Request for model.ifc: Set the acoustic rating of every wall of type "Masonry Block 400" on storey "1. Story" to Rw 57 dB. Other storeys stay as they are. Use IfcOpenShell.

First a look at what the model holds.

```python
import ifcopenshell
import ifcopenshell.util.element

model = ifcopenshell.open("model.ifc")
print(model.schema)
storey = next(s for s in model.by_type("IfcBuildingStorey") if s.Name == "1. Story")
walls = [e for e in ifcopenshell.util.element.get_decomposition(storey) if e.is_a("IfcWall")]
seen = {}
for e in walls:
    element_type = ifcopenshell.util.element.get_type(e)
    key = (element_type.Name if element_type != e and element_type else None, ifcopenshell.util.element.get_pset(e, "Pset_WallCommon", "AcousticRating"))
    seen[key] = seen.get(key, 0) + 1
for (name, value), count in sorted(seen.items(), key=str):
    print(count, "x", name, "|", value)
```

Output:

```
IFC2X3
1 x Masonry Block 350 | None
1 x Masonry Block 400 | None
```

```python
import ifcopenshell
import ifcopenshell.api.pset
import ifcopenshell.util.element

model = ifcopenshell.open("model.ifc")

storey = next(s for s in model.by_type("IfcBuildingStorey") if s.Name == "1. Story")
walls = [e for e in ifcopenshell.util.element.get_decomposition(storey) if e.is_a("IfcWall")]

count = 0
for e in walls:
    element_type = ifcopenshell.util.element.get_type(e)
    if element_type in (None, e) or element_type.Name != "Masonry Block 400":
        continue
    # add_pset returns the element's existing set when there is one.
    pset = ifcopenshell.api.pset.add_pset(model, product=e, name="Pset_WallCommon")
    ifcopenshell.api.pset.edit_pset(model, pset=pset, properties={"AcousticRating": "Rw 57 dB"})
    count += 1

print(count, "walls updated")

model.write("model-out.ifc")
```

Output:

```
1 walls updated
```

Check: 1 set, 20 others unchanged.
